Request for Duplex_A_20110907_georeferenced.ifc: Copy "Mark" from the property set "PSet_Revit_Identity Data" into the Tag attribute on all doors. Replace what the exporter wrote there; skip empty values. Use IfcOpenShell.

First a look at what the model holds.

```python
import ifcopenshell
import ifcopenshell.util.element

model = ifcopenshell.open("Duplex_A_20110907_georeferenced.ifc")
print(model.schema)
doors = model.by_type("IfcDoor")
print(len(doors), "doors")
for e in doors[:8]:
    source = ifcopenshell.util.element.get_pset(e, "PSet_Revit_Identity Data", "Mark")
    target = e.Tag
    print(e.id(), repr(source), repr(target), sep=" | ")
```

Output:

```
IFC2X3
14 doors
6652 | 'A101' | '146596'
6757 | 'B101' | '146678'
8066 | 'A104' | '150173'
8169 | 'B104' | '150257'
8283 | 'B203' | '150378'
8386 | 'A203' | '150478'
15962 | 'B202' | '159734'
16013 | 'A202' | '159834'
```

```python
import ifcopenshell
import ifcopenshell.util.element

model = ifcopenshell.open("Duplex_A_20110907_georeferenced.ifc")

count = 0
for e in model.by_type("IfcDoor"):
    value = ifcopenshell.util.element.get_pset(e, "PSet_Revit_Identity Data", "Mark")
    current = e.Tag
    if not value or not value.strip() or current == value:
        continue
    e.Tag = value
    count += 1

print(count, "doors updated")

model.write("Duplex_A_20110907_georeferenced_edited.ifc")
```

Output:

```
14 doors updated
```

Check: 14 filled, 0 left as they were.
